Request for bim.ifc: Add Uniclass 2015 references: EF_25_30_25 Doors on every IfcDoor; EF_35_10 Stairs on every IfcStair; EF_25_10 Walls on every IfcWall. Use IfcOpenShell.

First a look at what the model holds.

```python
import ifcopenshell

model = ifcopenshell.open("bim.ifc")
print(model.schema)
print("classifications:", [c.Name for c in model.by_type("IfcClassification")])
for ifc_class in ("IfcDoor", "IfcRoof", "IfcStair", "IfcWall", "IfcWindow"):
    print(ifc_class, len(model.by_type(ifc_class)))
```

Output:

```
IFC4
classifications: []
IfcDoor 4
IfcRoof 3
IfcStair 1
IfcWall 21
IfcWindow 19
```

```python
import ifcopenshell
import ifcopenshell.api.classification

model = ifcopenshell.open("bim.ifc")

system = ifcopenshell.api.classification.add_classification(model, classification="Uniclass 2015")

codes = {
    "IfcDoor": ("EF_25_30_25", "Doors"),
    "IfcStair": ("EF_35_10", "Stairs"),
    "IfcWall": ("EF_25_10", "Walls"),
}
for ifc_class, (code, name) in codes.items():
    products = model.by_type(ifc_class)
    ifcopenshell.api.classification.add_reference(
        model, products=products, classification=system, identification=code, name=name
    )
    print(code, len(products))

model.write("bim_edited.ifc")
```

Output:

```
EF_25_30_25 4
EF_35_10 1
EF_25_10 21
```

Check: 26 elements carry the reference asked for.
